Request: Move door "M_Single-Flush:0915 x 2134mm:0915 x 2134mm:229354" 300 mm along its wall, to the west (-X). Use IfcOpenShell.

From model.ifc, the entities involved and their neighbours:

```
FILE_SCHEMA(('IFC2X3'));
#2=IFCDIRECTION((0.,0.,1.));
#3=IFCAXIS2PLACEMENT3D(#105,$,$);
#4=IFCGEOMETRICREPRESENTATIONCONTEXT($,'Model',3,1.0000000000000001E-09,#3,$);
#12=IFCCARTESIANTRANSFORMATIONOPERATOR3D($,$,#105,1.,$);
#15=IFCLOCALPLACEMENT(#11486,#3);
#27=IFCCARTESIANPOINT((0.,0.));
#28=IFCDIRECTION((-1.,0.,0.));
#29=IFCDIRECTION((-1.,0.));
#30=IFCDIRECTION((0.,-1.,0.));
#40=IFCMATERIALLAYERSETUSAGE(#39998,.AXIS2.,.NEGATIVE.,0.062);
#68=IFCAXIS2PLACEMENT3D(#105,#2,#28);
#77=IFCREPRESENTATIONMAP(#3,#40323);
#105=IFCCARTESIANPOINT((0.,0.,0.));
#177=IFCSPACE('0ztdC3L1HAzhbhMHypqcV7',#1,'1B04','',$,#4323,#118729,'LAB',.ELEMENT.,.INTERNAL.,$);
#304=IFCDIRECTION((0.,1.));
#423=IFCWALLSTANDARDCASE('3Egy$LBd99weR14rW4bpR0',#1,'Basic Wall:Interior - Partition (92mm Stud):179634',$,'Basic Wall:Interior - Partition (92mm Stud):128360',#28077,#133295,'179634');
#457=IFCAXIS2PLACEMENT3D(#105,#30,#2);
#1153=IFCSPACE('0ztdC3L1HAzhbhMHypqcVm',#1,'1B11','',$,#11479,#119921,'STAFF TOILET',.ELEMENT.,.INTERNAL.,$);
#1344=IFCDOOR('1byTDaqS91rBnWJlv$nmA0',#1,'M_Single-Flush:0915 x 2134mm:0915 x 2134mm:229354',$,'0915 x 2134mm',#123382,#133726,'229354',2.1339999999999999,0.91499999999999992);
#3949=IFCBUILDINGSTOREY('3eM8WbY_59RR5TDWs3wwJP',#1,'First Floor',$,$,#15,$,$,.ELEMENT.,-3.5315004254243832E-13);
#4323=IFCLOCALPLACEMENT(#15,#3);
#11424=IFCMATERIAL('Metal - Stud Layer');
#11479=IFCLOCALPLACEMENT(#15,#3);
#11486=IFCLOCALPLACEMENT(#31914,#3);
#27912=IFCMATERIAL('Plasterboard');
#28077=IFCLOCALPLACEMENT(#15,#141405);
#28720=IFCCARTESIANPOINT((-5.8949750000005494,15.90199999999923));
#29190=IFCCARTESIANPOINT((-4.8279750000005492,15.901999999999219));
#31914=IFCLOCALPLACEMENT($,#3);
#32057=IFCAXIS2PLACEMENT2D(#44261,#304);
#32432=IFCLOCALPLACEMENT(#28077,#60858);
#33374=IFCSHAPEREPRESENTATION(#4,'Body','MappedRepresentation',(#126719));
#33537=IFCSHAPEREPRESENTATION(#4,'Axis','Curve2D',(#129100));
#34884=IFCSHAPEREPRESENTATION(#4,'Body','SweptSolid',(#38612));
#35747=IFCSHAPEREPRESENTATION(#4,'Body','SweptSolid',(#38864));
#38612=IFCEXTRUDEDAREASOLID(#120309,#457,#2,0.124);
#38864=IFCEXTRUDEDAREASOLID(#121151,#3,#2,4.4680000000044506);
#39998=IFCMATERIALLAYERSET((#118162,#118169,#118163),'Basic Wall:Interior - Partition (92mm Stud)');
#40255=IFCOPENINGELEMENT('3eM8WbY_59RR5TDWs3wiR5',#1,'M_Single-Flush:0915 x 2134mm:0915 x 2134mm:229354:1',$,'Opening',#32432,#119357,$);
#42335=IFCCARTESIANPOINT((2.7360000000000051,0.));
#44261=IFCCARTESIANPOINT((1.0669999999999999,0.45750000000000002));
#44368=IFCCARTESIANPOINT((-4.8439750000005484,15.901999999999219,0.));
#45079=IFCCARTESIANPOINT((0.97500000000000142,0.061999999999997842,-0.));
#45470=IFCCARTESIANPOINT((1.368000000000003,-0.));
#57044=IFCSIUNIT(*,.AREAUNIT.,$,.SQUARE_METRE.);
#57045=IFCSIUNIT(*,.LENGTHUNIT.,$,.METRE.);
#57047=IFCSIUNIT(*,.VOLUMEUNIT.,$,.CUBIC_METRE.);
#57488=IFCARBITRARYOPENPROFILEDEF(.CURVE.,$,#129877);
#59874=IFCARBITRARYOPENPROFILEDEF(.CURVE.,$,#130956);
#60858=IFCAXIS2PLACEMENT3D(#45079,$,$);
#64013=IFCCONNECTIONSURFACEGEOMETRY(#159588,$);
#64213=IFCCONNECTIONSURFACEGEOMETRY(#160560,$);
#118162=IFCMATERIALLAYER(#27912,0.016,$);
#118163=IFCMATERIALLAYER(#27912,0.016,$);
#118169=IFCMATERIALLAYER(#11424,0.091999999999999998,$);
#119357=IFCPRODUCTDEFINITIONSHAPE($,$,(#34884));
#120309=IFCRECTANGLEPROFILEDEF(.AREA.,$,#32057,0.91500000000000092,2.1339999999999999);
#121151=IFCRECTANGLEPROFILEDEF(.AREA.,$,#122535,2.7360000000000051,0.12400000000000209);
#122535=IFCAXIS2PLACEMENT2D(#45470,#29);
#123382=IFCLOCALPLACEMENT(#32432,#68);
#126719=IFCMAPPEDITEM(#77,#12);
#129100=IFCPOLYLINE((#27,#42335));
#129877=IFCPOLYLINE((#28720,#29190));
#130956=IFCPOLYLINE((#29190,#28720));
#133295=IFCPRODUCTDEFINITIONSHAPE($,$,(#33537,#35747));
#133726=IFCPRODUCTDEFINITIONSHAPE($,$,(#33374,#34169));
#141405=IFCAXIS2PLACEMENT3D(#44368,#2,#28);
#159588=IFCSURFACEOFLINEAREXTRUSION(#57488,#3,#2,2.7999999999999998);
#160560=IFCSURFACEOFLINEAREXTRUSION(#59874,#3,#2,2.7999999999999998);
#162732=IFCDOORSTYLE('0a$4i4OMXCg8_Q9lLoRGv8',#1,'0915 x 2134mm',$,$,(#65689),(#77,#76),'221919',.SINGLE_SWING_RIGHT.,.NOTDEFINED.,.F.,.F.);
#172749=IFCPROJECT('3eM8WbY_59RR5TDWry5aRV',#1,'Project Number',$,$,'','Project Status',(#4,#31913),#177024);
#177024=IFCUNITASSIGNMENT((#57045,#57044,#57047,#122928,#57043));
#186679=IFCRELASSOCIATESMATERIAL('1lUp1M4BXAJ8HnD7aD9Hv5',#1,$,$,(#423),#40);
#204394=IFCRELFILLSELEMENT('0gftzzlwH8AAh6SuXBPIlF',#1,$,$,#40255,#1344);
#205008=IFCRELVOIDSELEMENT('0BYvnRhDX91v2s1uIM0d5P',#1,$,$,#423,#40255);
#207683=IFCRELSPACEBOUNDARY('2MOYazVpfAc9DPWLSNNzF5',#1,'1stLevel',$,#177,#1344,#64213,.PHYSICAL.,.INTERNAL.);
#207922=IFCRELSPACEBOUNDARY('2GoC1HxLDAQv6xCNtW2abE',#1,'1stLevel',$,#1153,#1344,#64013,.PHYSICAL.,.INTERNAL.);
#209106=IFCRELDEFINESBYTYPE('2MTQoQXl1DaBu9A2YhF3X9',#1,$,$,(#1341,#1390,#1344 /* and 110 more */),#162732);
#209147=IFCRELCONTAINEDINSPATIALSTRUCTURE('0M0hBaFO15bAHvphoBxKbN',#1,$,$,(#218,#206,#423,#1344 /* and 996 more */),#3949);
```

```python
import numpy as np
import ifcopenshell
import ifcopenshell.api.geometry
import ifcopenshell.util.placement

model = ifcopenshell.open("model.ifc")

door = model.by_id(1344)
opening = door.FillsVoids[0].RelatingOpeningElement
wall = opening.VoidsElements[0].RelatingBuildingElement

wall_matrix = ifcopenshell.util.placement.get_local_placement(wall.ObjectPlacement)
shift = wall_matrix[:3, 0] * 0.3
before = ifcopenshell.util.placement.get_local_placement(door.ObjectPlacement)[:3, 3].copy()

# The door is placed relative to its opening, so it follows when the opening moves.
matrix = ifcopenshell.util.placement.get_local_placement(opening.ObjectPlacement)
matrix[:3, 3] += shift
ifcopenshell.api.geometry.edit_object_placement(
    model, product=opening, matrix=matrix, is_si=False, should_transform_children=True
)

# Space boundary surfaces are stored in each space's coordinates; move them too.
for rel in door.ProvidesBoundaries:
    if not rel.ConnectionGeometry:
        continue
    surface = rel.ConnectionGeometry.SurfaceOnRelatingElement
    space_matrix = ifcopenshell.util.placement.get_local_placement(rel.RelatingSpace.ObjectPlacement)
    point = np.array(surface.Position.Location.Coordinates) + space_matrix[:3, :3].T @ shift
    surface.Position = model.createIfcAxis2Placement3D(
        model.createIfcCartesianPoint(point.tolist()), surface.Position.Axis, surface.Position.RefDirection
    )

after = ifcopenshell.util.placement.get_local_placement(door.ObjectPlacement)[:3, 3]
print("door moved by", (after - before).round(3) + 0.0)

model.write("model_updated.ifc")
```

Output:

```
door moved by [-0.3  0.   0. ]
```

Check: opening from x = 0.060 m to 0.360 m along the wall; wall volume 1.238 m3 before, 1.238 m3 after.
